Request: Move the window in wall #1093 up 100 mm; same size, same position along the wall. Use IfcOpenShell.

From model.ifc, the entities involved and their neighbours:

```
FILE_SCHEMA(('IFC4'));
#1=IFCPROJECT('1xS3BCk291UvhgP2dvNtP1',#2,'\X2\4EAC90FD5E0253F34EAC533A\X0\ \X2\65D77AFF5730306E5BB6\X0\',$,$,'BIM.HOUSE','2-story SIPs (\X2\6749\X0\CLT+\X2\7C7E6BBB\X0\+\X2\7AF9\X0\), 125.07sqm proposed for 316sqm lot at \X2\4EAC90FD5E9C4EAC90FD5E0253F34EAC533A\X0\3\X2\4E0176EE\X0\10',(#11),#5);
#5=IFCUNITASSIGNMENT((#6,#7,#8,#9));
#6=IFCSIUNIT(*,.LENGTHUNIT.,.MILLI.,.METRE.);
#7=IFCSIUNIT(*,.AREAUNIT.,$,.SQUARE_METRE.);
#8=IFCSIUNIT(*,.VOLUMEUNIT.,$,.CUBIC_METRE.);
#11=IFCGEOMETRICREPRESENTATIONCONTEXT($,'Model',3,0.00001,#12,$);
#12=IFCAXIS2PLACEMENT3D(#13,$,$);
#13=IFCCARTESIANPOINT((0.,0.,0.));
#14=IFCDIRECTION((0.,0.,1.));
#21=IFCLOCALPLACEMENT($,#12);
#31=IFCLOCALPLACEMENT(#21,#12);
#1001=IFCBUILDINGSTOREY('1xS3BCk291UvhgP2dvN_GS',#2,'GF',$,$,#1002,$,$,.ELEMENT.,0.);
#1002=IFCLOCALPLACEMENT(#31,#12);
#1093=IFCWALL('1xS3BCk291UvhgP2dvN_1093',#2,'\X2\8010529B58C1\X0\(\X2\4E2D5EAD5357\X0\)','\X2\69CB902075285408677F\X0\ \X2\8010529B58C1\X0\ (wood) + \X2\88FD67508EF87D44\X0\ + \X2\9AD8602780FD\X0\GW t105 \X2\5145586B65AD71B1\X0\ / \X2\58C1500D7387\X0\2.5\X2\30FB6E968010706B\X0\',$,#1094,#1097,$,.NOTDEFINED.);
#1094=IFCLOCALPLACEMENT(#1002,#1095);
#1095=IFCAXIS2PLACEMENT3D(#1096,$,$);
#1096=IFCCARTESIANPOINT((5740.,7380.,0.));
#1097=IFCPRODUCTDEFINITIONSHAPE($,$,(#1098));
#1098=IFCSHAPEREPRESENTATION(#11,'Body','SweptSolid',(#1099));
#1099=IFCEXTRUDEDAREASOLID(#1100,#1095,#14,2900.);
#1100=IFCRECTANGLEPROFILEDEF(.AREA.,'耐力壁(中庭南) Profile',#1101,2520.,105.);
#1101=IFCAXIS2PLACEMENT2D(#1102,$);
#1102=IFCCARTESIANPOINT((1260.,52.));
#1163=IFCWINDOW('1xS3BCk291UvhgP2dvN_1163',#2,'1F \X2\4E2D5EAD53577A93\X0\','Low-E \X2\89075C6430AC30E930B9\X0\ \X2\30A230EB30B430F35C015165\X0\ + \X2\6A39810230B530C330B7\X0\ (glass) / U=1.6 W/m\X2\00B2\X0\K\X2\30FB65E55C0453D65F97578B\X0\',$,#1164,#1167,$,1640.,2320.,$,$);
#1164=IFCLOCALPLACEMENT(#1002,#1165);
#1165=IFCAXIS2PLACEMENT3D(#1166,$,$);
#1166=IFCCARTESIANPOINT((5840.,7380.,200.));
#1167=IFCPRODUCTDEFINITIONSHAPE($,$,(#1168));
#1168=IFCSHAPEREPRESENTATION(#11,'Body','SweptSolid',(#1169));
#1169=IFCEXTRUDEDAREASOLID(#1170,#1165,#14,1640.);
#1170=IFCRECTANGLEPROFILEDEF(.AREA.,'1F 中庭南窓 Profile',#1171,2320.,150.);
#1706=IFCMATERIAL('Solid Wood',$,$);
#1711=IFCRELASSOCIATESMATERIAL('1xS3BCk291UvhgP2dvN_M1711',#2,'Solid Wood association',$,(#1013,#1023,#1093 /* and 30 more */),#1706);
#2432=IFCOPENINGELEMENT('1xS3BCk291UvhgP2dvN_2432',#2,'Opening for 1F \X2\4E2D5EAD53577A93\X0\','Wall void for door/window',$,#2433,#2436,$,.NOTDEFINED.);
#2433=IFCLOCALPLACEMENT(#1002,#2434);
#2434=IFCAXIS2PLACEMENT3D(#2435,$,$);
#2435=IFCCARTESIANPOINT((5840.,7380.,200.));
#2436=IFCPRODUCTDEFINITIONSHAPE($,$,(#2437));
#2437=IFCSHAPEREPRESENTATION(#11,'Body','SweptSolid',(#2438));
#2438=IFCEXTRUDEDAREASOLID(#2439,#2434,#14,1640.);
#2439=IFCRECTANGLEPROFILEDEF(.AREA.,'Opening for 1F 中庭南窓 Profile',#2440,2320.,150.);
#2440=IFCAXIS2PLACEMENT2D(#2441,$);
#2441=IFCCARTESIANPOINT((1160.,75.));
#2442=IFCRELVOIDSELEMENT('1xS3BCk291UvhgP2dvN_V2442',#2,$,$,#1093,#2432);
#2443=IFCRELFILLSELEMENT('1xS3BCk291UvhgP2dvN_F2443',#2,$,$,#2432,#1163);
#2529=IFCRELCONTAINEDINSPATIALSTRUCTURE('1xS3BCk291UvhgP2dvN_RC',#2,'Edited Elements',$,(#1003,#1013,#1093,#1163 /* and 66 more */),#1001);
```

```python
import numpy as np
import ifcopenshell
import ifcopenshell.api.geometry
import ifcopenshell.util.placement
import ifcopenshell.util.unit

model = ifcopenshell.open("model.ifc")
unit_scale = ifcopenshell.util.unit.calculate_unit_scale(model)

window = model.by_guid("1xS3BCk291UvhgP2dvN_1163")
opening = window.FillsVoids[0].RelatingOpeningElement
dz = 0.1 / unit_scale

shift = np.array([0.0, 0.0, dz])
# The window is not placed relative to its opening, so move both.
for product in (opening, window):
    matrix = ifcopenshell.util.placement.get_local_placement(product.ObjectPlacement)
    matrix[:3, 3] += shift
    ifcopenshell.api.geometry.edit_object_placement(model, product=product, matrix=matrix, is_si=False)

print(f"moved by {dz * unit_scale:+.3f} m")

model.write("model_v2.ifc")
```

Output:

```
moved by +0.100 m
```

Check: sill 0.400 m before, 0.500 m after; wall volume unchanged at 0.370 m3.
